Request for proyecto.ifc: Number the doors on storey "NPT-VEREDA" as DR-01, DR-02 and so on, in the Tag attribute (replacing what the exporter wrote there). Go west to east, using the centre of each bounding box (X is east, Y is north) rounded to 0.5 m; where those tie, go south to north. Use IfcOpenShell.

First a look at what the model holds.

```python
import ifcopenshell
import ifcopenshell.util.element
import ifcopenshell.util.placement

model = ifcopenshell.open("proyecto.ifc")
print(model.schema)
storey = next(s for s in model.by_type("IfcBuildingStorey") if s.Name == "NPT-VEREDA")
doors = [e for e in ifcopenshell.util.element.get_decomposition(storey) if e.is_a("IfcDoor")]
for e in sorted(doors, key=lambda e: e.id()):
    origin = ifcopenshell.util.placement.get_local_placement(e.ObjectPlacement)[:3, 3]
    print(e.id(), e.Tag, e.Name, origin.round(2) + 0.0, sep=" | ")
```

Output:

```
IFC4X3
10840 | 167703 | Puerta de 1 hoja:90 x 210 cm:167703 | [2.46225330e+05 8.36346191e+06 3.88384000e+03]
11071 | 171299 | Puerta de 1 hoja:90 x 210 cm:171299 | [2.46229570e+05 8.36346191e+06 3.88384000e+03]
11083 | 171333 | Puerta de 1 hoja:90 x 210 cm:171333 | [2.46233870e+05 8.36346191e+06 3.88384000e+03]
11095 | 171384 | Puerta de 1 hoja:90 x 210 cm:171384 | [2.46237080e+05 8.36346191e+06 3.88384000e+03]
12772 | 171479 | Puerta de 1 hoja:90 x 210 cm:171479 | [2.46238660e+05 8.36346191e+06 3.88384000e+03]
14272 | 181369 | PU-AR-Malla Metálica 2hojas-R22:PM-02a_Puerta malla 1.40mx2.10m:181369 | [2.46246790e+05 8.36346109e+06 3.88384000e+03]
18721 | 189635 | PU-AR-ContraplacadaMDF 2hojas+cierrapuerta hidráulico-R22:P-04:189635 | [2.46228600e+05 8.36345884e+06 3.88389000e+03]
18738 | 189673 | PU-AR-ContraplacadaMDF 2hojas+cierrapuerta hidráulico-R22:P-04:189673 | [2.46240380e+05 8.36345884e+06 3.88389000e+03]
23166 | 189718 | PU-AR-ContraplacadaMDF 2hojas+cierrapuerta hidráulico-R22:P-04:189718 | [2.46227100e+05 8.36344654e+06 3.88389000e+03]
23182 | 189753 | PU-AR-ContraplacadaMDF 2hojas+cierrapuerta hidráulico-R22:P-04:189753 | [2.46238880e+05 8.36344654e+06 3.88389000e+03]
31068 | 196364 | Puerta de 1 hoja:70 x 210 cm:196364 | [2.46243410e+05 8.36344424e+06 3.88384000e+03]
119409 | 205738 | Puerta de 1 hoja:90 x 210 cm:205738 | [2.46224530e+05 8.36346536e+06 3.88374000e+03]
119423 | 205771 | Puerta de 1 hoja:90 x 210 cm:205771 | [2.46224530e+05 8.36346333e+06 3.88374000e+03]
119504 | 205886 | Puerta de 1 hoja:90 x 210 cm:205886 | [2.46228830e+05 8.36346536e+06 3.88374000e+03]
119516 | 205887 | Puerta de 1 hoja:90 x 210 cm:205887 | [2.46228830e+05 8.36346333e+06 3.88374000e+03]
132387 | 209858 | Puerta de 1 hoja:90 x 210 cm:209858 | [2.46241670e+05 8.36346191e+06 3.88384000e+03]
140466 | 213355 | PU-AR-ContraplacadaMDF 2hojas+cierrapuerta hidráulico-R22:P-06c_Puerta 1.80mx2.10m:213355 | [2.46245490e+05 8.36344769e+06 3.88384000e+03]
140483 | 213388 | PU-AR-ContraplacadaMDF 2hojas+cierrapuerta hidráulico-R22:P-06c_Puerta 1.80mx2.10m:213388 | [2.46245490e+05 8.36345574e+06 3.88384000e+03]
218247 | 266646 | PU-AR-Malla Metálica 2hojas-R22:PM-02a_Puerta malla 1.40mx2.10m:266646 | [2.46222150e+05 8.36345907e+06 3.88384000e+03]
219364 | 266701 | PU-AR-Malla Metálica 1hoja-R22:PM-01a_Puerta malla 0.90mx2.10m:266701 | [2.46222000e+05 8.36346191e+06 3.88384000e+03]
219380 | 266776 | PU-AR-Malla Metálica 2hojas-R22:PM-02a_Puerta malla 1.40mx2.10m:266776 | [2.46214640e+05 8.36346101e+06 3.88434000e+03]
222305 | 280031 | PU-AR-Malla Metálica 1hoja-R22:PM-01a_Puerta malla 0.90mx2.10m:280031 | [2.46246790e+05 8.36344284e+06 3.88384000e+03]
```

```python
import ifcopenshell
import ifcopenshell.geom
import ifcopenshell.util.element
import ifcopenshell.util.shape

model = ifcopenshell.open("proyecto.ifc")
settings = ifcopenshell.geom.settings()
settings.set("use-world-coords", True)


def centre(element):
    shape = ifcopenshell.geom.create_shape(settings, element)
    return ifcopenshell.util.shape.get_bbox_centroid(shape.geometry)


storey = next(s for s in model.by_type("IfcBuildingStorey") if s.Name == "NPT-VEREDA")
doors = [e for e in ifcopenshell.util.element.get_decomposition(storey) if e.is_a("IfcDoor")]

# Insertion points can sit at a corner or the storey origin, so sort by the geometry (in metres).
centres = {e: centre(e) for e in doors}
doors.sort(key=lambda e: (round(centres[e][0] / 0.5), centres[e][1]))

for i, e in enumerate(doors, start=1):
    number = f"DR-{i:02d}"
    e.Tag = number
    print(e.id(), number)

model.write("proyecto-out.ifc")
```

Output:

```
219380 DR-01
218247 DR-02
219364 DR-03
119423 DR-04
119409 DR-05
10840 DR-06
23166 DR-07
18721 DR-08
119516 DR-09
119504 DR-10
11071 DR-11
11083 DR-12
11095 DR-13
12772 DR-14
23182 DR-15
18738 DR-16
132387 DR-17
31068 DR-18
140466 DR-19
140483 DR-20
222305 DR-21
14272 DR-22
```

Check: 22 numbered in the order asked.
